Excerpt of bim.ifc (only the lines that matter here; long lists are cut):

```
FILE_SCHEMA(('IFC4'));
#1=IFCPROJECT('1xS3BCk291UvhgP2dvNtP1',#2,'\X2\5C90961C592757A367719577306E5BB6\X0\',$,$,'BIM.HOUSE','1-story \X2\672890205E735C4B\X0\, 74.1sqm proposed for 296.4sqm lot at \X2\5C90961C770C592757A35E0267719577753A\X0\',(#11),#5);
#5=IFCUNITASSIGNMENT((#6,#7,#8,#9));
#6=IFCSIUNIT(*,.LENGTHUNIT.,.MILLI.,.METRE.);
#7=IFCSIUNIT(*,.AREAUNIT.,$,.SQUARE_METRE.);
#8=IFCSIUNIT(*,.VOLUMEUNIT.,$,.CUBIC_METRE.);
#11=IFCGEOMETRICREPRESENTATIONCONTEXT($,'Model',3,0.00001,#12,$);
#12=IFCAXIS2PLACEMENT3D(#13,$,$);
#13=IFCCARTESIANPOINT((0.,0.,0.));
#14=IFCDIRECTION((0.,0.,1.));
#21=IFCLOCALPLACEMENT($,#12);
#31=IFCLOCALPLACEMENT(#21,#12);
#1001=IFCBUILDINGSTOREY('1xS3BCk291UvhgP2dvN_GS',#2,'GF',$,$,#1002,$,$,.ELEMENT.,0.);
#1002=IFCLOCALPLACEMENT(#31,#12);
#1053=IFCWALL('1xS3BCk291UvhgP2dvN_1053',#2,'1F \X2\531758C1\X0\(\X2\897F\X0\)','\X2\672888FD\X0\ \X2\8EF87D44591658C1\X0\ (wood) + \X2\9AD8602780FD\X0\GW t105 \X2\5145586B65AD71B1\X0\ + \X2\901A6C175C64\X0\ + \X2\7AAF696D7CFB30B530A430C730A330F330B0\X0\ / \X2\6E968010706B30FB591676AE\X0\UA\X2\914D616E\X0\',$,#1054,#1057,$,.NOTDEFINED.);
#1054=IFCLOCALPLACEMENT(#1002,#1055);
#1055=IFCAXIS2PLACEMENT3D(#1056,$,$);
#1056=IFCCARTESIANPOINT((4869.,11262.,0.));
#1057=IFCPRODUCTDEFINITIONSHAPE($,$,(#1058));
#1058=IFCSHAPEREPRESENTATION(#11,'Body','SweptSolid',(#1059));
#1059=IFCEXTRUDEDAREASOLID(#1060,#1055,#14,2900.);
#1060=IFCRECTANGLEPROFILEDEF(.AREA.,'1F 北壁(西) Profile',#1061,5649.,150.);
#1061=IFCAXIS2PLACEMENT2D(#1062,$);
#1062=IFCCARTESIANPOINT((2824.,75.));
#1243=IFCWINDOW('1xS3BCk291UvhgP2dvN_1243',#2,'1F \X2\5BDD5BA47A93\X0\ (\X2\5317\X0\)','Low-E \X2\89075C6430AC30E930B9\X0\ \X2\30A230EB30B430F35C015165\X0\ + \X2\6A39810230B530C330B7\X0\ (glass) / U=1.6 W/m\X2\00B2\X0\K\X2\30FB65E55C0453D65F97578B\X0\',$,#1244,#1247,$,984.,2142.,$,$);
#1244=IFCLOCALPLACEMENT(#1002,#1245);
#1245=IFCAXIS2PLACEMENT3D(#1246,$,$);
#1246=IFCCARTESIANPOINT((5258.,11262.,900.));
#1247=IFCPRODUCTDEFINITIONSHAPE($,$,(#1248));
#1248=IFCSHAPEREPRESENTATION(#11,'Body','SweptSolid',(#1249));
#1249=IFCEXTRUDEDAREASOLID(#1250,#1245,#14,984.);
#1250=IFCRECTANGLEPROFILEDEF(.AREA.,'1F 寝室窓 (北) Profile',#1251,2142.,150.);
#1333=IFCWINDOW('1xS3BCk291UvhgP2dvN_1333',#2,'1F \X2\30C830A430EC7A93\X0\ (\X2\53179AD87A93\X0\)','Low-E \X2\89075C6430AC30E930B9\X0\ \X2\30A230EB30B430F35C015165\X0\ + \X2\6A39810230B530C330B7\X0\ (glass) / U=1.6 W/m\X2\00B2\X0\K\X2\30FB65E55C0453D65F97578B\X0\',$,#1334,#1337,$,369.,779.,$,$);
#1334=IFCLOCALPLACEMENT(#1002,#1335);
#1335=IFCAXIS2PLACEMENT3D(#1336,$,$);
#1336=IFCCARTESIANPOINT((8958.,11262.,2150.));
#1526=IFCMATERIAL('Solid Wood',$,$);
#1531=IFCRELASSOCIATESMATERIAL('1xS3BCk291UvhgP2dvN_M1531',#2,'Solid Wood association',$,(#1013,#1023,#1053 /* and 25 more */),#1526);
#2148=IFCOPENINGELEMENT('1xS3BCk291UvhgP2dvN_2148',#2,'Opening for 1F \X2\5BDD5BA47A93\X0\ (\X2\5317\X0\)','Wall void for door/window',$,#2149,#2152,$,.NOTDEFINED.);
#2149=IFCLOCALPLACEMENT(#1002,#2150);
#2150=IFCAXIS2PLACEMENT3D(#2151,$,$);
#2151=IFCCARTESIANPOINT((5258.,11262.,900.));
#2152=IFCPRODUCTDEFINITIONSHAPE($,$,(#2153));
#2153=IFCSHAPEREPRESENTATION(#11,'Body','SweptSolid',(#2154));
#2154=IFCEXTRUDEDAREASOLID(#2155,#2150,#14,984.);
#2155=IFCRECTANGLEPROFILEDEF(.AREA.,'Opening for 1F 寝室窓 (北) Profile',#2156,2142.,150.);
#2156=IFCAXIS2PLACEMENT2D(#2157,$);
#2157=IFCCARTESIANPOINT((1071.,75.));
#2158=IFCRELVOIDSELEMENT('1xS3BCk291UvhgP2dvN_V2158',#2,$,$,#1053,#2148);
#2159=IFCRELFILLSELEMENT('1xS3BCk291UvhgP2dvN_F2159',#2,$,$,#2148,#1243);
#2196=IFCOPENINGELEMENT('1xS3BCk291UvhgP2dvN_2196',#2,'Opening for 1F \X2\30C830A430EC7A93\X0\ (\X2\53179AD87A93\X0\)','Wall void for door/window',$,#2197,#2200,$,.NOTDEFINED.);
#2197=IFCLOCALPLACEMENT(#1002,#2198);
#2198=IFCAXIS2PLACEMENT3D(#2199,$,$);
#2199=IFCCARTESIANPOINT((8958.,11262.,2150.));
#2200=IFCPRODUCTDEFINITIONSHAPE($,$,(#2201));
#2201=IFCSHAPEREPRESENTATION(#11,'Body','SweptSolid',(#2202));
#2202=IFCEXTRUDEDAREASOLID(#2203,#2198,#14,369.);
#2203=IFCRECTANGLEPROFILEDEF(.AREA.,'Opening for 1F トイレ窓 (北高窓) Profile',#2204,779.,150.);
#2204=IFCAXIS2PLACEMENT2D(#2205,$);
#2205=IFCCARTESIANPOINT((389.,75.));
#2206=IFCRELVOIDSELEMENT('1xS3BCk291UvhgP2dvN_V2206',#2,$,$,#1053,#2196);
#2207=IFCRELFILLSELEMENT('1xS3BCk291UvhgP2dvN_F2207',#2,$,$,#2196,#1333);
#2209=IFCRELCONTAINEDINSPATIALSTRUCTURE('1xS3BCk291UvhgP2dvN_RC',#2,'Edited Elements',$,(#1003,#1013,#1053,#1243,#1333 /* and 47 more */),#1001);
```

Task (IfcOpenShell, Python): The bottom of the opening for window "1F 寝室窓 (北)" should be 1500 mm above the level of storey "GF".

```python
import numpy as np
import ifcopenshell
import ifcopenshell.api.geometry
import ifcopenshell.geom
import ifcopenshell.util.element
import ifcopenshell.util.placement
import ifcopenshell.util.shape
import ifcopenshell.util.unit

model = ifcopenshell.open("bim.ifc")
unit_scale = ifcopenshell.util.unit.calculate_unit_scale(model)

window = model.by_guid("1xS3BCk291UvhgP2dvN_1243")
opening = window.FillsVoids[0].RelatingOpeningElement
storey = ifcopenshell.util.element.get_container(window, ifc_class="IfcBuildingStorey")
level = ifcopenshell.util.placement.get_local_placement(storey.ObjectPlacement)[2, 3]

# The opening's origin need not be at the sill, so measure its lowest point.
shape = ifcopenshell.geom.create_shape(ifcopenshell.geom.settings(), opening)
bottom = ifcopenshell.util.shape.get_shape_bottom_elevation(shape, shape.geometry) / unit_scale
dz = level + 1.5 / unit_scale - bottom

shift = np.array([0.0, 0.0, dz])
# The window is not placed relative to its opening, so move both.
for product in (opening, window):
    matrix = ifcopenshell.util.placement.get_local_placement(product.ObjectPlacement)
    matrix[:3, 3] += shift
    ifcopenshell.api.geometry.edit_object_placement(model, product=product, matrix=matrix, is_si=False)

print(f"moved by {dz * unit_scale:+.3f} m")

model.write("bim_rev.ifc")
```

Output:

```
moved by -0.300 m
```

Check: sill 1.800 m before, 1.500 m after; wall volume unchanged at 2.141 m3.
